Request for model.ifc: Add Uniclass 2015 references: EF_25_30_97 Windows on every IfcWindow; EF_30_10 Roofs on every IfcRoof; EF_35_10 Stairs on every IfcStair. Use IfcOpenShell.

First a look at what the model holds.

```python
import ifcopenshell

model = ifcopenshell.open("model.ifc")
print(model.schema)
print("classifications:", [c.Name for c in model.by_type("IfcClassification")])
for ifc_class in ("IfcDoor", "IfcRoof", "IfcStair", "IfcWall", "IfcWindow"):
    print(ifc_class, len(model.by_type(ifc_class)))
```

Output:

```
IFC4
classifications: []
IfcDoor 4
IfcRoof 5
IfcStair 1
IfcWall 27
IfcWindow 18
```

```python
import ifcopenshell
import ifcopenshell.api.classification

model = ifcopenshell.open("model.ifc")

system = ifcopenshell.api.classification.add_classification(model, classification="Uniclass 2015")

codes = {
    "IfcWindow": ("EF_25_30_97", "Windows"),
    "IfcRoof": ("EF_30_10", "Roofs"),
    "IfcStair": ("EF_35_10", "Stairs"),
}
for ifc_class, (code, name) in codes.items():
    products = model.by_type(ifc_class)
    ifcopenshell.api.classification.add_reference(
        model, products=products, classification=system, identification=code, name=name
    )
    print(code, len(products))

model.write("model_v2.ifc")
```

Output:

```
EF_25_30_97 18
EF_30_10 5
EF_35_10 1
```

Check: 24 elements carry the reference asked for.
